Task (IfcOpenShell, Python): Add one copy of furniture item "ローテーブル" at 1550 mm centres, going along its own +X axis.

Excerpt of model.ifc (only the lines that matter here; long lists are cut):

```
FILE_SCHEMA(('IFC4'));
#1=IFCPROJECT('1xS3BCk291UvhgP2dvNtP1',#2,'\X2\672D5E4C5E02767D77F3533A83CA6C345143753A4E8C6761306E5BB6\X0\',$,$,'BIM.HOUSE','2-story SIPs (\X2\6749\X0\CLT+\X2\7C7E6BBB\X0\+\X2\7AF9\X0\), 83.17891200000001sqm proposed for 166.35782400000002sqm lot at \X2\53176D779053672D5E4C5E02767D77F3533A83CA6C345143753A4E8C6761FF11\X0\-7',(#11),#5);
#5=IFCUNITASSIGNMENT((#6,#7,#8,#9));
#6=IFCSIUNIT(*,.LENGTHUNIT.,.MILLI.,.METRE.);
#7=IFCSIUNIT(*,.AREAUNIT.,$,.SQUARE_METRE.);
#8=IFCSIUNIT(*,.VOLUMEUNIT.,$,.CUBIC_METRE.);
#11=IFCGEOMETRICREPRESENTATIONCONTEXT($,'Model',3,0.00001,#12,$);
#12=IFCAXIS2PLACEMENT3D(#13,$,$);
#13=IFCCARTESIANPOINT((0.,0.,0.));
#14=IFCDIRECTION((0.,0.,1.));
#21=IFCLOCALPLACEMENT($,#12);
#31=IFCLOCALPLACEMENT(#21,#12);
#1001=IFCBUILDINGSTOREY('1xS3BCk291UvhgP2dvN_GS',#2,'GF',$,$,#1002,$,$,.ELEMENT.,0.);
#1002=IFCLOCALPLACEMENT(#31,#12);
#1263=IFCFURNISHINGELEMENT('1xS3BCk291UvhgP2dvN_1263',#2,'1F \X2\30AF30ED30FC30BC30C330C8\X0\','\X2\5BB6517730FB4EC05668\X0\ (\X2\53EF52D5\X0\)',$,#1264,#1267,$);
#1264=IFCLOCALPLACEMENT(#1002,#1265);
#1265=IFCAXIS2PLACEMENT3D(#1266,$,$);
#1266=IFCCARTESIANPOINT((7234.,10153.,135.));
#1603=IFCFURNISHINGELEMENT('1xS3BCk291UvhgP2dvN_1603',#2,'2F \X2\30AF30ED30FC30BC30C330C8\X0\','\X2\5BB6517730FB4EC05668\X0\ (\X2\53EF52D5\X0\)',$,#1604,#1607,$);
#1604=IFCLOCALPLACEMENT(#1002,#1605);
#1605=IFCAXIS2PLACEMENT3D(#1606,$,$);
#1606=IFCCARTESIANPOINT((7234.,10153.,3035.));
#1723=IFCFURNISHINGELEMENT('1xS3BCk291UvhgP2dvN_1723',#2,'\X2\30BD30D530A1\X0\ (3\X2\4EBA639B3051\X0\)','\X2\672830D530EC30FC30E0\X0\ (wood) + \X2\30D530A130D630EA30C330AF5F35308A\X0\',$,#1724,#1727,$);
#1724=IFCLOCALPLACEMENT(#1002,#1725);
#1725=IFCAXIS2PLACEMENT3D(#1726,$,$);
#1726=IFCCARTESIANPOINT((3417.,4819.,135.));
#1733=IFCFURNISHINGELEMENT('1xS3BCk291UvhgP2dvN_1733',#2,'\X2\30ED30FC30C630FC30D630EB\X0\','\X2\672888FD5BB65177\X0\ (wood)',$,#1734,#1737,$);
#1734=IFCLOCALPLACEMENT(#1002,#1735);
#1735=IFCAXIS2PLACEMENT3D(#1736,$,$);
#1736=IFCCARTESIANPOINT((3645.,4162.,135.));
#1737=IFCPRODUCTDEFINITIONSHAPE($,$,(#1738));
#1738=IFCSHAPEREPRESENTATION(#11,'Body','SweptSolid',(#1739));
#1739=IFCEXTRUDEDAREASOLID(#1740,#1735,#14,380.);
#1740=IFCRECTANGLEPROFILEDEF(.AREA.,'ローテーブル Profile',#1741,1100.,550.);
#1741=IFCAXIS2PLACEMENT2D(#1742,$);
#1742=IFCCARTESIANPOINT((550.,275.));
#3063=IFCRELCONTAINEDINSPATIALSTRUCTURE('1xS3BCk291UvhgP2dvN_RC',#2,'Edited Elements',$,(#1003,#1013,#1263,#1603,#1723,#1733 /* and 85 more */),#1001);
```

```python
import ifcopenshell
import ifcopenshell.api.geometry
import ifcopenshell.api.root
import ifcopenshell.util.element
import ifcopenshell.util.placement

model = ifcopenshell.open("model.ifc")


def reuse_history(source, copy):
    """copy_class also copies each property set's owner history, people and application; keep the originals."""
    for rel in copy.IsDefinedBy:
        if rel.is_a("IfcRelDefinesByProperties") and (history := rel.RelatingPropertyDefinition.OwnerHistory):
            rel.RelatingPropertyDefinition.OwnerHistory = source.OwnerHistory
            ifcopenshell.util.element.remove_deep2(model, history)


source = model.by_guid("1xS3BCk291UvhgP2dvN_1733")
base = ifcopenshell.util.placement.get_local_placement(source.ObjectPlacement)
step = base[:3, 0] * 1550.0

for i in range(1, 2):
    copy = ifcopenshell.api.root.copy_class(model, product=source)
    copy.Representation = ifcopenshell.util.element.copy_deep(
        model, source.Representation, exclude=["IfcGeometricRepresentationContext", "IfcRepresentationMap"]
    )
    reuse_history(source, copy)
    matrix = base.copy()
    matrix[:3, 3] += i * step
    print("added at", matrix[:3, 3].round(3) + 0.0)
    ifcopenshell.api.geometry.edit_object_placement(model, product=copy, matrix=matrix, is_si=False)

model.write("model-out.ifc")
```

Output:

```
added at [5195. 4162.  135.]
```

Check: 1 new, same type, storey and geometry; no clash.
